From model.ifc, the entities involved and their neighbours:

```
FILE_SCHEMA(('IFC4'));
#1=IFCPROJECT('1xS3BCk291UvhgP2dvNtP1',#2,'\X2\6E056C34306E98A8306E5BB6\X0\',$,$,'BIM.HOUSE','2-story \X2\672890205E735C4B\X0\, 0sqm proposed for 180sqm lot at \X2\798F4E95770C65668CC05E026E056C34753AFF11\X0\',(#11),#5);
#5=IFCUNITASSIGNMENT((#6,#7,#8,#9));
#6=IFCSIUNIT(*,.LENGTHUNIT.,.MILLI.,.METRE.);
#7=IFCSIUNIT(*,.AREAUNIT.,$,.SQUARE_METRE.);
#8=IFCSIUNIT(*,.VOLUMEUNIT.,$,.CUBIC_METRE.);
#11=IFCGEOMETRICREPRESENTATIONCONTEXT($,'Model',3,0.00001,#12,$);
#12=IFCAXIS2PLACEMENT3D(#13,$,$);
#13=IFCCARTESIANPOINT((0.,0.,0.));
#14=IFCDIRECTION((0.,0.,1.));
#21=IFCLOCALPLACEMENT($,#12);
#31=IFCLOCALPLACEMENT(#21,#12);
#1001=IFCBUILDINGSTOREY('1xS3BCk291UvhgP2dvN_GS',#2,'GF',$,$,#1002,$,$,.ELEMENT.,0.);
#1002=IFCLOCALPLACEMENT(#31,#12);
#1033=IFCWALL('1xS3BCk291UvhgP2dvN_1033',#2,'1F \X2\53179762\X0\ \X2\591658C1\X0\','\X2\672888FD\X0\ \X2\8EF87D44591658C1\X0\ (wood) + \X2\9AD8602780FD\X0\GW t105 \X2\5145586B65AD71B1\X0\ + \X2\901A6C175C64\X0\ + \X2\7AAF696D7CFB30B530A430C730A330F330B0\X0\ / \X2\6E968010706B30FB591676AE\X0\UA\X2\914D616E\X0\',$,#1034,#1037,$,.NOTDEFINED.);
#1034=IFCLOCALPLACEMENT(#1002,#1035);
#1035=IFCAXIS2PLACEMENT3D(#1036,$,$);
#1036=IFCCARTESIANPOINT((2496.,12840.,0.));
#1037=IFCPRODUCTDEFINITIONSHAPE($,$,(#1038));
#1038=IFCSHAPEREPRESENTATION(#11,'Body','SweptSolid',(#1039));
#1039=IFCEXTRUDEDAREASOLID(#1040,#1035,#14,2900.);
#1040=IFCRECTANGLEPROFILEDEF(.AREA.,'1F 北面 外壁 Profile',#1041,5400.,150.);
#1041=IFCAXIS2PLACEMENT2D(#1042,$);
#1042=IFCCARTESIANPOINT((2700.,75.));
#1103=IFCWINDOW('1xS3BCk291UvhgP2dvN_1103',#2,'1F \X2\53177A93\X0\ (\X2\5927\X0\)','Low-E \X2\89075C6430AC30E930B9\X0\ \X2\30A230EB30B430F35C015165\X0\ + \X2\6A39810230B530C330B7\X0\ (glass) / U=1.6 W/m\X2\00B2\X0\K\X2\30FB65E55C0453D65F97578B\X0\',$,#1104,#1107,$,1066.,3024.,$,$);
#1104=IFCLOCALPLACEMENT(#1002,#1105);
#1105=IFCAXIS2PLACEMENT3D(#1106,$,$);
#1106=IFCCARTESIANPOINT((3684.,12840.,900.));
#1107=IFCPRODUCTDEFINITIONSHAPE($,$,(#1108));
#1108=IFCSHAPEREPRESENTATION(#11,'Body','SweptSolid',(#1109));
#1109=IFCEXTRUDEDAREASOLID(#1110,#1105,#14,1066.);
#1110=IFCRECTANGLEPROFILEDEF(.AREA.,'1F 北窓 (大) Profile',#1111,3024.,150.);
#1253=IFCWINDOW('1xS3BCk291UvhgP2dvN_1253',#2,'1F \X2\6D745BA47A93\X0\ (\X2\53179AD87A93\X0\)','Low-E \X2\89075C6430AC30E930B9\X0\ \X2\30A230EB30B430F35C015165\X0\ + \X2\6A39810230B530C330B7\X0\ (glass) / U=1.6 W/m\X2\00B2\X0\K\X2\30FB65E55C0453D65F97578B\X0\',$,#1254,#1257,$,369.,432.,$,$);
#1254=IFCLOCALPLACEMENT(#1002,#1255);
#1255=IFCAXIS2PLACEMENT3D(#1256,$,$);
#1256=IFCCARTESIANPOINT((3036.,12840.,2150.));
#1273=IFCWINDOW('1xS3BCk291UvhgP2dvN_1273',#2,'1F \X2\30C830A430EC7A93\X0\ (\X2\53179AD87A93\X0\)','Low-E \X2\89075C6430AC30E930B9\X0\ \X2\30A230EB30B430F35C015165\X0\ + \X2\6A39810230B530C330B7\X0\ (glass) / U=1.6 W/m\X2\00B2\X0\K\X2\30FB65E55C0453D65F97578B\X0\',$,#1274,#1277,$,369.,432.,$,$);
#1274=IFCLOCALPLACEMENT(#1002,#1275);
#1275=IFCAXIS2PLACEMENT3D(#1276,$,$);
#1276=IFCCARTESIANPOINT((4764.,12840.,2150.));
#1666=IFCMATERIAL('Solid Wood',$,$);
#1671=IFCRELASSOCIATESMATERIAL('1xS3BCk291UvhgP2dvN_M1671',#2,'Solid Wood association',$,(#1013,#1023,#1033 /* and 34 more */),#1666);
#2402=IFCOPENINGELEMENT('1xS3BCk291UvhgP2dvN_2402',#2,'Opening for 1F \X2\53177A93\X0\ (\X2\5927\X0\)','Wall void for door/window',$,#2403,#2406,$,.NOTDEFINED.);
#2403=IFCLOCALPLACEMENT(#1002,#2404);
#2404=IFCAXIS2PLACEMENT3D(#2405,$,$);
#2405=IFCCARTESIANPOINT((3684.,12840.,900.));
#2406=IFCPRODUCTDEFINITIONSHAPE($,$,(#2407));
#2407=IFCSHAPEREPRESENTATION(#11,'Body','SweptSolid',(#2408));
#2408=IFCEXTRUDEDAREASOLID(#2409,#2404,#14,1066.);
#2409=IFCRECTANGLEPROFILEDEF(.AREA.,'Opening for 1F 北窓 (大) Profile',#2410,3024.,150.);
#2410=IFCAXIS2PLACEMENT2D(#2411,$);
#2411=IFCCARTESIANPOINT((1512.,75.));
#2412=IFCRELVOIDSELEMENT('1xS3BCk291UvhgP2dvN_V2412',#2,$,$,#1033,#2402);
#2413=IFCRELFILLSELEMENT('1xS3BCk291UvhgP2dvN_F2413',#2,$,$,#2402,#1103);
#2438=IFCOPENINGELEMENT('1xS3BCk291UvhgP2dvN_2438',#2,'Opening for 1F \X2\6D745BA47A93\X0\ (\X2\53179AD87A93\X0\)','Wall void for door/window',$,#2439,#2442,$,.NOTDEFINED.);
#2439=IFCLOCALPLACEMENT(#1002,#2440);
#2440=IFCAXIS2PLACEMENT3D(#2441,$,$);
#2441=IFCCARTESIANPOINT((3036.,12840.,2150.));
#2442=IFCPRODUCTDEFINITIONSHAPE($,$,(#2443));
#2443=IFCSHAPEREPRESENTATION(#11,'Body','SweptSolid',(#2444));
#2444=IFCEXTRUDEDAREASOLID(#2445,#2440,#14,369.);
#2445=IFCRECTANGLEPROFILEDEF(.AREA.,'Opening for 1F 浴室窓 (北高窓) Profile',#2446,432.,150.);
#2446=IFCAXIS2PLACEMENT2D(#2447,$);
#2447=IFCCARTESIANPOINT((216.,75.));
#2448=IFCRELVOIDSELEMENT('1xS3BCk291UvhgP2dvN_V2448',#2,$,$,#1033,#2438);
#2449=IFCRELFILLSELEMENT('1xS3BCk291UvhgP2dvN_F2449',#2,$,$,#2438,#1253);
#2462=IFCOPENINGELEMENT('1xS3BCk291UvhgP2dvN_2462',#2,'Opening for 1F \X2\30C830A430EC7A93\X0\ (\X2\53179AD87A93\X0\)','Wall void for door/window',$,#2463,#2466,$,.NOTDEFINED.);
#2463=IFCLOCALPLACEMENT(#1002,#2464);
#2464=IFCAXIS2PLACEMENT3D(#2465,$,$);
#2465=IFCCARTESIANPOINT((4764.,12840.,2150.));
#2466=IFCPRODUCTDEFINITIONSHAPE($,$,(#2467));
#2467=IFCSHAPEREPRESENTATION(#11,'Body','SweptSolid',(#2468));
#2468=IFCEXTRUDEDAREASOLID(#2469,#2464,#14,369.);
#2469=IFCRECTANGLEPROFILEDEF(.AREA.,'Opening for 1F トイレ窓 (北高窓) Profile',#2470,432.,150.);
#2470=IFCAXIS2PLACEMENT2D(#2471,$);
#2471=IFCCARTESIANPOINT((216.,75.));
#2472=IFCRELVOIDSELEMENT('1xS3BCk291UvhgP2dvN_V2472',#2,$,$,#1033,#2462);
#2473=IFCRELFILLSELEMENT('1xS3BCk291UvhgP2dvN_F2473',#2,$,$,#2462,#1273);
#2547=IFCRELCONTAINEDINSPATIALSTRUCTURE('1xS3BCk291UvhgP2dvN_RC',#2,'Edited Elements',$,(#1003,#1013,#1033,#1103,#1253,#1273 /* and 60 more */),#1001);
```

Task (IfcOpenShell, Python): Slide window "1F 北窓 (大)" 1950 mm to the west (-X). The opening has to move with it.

```python
import ifcopenshell
import ifcopenshell.api.geometry
import ifcopenshell.util.placement

model = ifcopenshell.open("model.ifc")

window = model.by_guid("1xS3BCk291UvhgP2dvN_1103")
opening = window.FillsVoids[0].RelatingOpeningElement
wall = opening.VoidsElements[0].RelatingBuildingElement

wall_matrix = ifcopenshell.util.placement.get_local_placement(wall.ObjectPlacement)
shift = wall_matrix[:3, 0] * -1950.0
before = ifcopenshell.util.placement.get_local_placement(window.ObjectPlacement)[:3, 3].copy()

# The window is not placed relative to its opening, so move both.
for product in (opening, window):
    matrix = ifcopenshell.util.placement.get_local_placement(product.ObjectPlacement)
    matrix[:3, 3] += shift
    ifcopenshell.api.geometry.edit_object_placement(model, product=product, matrix=matrix, is_si=False)

after = ifcopenshell.util.placement.get_local_placement(window.ObjectPlacement)[:3, 3]
print("window moved by", (after - before).round(3) + 0.0)

model.write("model_edited.ifc")
```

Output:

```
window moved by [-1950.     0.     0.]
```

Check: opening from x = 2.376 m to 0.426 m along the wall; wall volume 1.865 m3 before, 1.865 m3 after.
